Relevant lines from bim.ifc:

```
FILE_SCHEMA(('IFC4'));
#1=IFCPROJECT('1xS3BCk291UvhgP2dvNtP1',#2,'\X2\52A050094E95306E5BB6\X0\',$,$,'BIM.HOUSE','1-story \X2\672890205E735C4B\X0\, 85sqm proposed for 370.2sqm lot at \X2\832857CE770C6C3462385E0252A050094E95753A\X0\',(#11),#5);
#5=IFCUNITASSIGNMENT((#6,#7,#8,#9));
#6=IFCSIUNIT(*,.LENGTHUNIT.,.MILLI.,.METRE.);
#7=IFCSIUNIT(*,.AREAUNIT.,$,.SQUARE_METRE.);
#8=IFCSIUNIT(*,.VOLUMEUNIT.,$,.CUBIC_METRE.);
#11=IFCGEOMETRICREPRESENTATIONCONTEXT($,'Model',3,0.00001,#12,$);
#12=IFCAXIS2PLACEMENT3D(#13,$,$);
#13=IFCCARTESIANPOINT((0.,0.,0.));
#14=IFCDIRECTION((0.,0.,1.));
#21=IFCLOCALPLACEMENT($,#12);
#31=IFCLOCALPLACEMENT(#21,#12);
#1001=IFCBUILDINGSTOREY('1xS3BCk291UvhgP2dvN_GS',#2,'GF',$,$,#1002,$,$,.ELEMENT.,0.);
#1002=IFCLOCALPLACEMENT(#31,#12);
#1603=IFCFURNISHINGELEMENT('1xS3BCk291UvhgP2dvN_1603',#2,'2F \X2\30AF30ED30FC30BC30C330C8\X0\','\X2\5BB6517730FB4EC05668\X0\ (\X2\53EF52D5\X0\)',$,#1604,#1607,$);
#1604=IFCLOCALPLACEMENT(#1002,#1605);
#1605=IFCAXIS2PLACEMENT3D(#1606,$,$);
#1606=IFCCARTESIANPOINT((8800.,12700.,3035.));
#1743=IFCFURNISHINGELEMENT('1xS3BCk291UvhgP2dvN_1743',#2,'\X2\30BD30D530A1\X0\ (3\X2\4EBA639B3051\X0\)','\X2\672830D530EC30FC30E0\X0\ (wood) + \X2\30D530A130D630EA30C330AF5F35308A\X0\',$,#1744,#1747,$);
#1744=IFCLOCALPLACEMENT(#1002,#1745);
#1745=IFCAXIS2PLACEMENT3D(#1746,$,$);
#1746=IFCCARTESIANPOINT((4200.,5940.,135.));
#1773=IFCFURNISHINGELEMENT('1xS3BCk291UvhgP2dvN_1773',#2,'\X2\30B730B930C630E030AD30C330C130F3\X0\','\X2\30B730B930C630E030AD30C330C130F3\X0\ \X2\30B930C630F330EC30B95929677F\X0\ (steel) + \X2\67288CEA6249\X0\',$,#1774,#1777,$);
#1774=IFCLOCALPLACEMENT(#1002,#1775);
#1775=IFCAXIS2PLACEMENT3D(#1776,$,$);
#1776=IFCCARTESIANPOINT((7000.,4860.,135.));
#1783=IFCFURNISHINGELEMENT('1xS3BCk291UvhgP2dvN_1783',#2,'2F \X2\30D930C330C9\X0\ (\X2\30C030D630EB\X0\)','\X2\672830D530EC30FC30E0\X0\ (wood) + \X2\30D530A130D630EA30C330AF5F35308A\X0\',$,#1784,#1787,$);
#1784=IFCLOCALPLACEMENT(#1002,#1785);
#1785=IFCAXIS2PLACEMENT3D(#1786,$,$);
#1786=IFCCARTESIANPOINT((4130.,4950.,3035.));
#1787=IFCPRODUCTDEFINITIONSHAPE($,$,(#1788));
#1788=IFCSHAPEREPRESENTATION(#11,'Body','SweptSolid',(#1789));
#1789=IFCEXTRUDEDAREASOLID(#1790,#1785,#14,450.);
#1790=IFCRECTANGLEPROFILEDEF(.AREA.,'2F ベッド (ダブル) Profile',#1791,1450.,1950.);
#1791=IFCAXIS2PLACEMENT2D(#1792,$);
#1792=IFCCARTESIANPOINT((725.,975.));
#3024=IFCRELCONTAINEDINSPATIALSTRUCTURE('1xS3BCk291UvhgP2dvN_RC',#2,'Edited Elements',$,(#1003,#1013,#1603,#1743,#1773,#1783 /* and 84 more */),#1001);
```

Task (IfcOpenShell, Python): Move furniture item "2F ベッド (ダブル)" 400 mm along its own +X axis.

```python
import ifcopenshell
import ifcopenshell.api.geometry
import ifcopenshell.util.placement

model = ifcopenshell.open("bim.ifc")

item = model.by_guid("1xS3BCk291UvhgP2dvN_1783")
matrix = ifcopenshell.util.placement.get_local_placement(item.ObjectPlacement)
matrix[:3, 3] += matrix[:3, 0] * 400.0
ifcopenshell.api.geometry.edit_object_placement(model, product=item, matrix=matrix, is_si=False)

print(ifcopenshell.util.placement.get_local_placement(item.ObjectPlacement).round(3) + 0.0)

model.write("bim-out.ifc")
```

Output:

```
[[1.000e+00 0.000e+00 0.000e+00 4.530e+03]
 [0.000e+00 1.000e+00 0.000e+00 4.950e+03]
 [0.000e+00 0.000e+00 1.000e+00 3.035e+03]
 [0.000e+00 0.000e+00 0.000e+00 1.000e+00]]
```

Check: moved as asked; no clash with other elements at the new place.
